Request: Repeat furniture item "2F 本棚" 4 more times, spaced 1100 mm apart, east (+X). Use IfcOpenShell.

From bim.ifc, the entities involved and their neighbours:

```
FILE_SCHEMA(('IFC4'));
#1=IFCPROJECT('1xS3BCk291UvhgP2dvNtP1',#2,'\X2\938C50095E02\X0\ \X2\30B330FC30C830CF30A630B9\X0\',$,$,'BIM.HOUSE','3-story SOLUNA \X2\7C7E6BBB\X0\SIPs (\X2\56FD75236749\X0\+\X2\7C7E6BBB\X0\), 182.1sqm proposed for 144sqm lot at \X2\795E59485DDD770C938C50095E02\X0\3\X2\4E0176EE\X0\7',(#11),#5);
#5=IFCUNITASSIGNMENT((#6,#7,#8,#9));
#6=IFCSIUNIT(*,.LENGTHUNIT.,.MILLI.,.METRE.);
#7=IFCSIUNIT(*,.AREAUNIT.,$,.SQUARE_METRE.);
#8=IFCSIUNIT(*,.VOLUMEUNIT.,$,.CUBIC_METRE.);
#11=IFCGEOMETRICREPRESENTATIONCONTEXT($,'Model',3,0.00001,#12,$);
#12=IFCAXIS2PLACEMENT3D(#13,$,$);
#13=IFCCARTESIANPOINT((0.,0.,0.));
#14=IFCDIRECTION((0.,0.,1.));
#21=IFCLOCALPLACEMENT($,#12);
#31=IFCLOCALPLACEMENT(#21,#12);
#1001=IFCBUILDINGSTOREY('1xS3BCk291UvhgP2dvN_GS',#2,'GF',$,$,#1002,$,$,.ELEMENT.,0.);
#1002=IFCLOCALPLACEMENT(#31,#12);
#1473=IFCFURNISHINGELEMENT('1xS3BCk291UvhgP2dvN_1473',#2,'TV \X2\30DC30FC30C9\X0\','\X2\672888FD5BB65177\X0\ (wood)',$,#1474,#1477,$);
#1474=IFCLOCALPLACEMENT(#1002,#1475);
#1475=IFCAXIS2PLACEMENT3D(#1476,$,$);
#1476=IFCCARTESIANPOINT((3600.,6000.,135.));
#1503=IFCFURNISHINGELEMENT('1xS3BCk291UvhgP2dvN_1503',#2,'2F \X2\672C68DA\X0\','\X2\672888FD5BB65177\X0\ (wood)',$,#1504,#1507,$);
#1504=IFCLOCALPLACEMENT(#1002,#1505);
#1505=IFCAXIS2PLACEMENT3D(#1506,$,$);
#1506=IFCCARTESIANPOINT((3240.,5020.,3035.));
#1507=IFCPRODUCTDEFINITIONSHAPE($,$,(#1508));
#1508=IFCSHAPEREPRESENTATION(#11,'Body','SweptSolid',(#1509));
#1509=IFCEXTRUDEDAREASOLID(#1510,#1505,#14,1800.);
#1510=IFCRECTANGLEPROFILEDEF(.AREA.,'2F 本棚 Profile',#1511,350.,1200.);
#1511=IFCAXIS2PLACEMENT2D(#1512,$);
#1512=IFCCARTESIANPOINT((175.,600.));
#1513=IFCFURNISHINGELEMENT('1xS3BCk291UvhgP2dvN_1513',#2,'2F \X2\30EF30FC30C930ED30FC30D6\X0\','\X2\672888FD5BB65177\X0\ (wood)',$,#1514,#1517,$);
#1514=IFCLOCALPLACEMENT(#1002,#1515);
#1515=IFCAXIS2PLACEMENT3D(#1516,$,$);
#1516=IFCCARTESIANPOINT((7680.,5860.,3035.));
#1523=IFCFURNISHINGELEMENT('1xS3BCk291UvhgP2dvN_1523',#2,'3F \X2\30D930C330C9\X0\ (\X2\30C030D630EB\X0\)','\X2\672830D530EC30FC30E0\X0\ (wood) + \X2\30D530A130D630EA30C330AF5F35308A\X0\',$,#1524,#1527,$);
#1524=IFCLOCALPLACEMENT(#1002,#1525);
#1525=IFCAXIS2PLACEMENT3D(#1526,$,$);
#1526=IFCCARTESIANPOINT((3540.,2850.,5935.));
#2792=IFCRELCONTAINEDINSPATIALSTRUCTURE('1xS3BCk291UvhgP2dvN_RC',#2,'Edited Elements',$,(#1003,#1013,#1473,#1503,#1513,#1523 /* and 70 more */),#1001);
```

```python
import numpy as np
import ifcopenshell
import ifcopenshell.api.geometry
import ifcopenshell.api.root
import ifcopenshell.util.element
import ifcopenshell.util.placement

model = ifcopenshell.open("bim.ifc")


def reuse_history(source, copy):
    """copy_class also copies each property set's owner history, people and application; keep the originals."""
    for rel in copy.IsDefinedBy:
        if rel.is_a("IfcRelDefinesByProperties") and (history := rel.RelatingPropertyDefinition.OwnerHistory):
            rel.RelatingPropertyDefinition.OwnerHistory = source.OwnerHistory
            ifcopenshell.util.element.remove_deep2(model, history)


source = model.by_guid("1xS3BCk291UvhgP2dvN_1503")
base = ifcopenshell.util.placement.get_local_placement(source.ObjectPlacement)
step = np.array([1.0, 0.0, 0.0]) * 1100.0

for i in range(1, 5):
    copy = ifcopenshell.api.root.copy_class(model, product=source)
    copy.Representation = ifcopenshell.util.element.copy_deep(
        model, source.Representation, exclude=["IfcGeometricRepresentationContext", "IfcRepresentationMap"]
    )
    reuse_history(source, copy)
    matrix = base.copy()
    matrix[:3, 3] += i * step
    print("added at", matrix[:3, 3].round(3) + 0.0)
    ifcopenshell.api.geometry.edit_object_placement(model, product=copy, matrix=matrix, is_si=False)

model.write("bim_rev.ifc")
```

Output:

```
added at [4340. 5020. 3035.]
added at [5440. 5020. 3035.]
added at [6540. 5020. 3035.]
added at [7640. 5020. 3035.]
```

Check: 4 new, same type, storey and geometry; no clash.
